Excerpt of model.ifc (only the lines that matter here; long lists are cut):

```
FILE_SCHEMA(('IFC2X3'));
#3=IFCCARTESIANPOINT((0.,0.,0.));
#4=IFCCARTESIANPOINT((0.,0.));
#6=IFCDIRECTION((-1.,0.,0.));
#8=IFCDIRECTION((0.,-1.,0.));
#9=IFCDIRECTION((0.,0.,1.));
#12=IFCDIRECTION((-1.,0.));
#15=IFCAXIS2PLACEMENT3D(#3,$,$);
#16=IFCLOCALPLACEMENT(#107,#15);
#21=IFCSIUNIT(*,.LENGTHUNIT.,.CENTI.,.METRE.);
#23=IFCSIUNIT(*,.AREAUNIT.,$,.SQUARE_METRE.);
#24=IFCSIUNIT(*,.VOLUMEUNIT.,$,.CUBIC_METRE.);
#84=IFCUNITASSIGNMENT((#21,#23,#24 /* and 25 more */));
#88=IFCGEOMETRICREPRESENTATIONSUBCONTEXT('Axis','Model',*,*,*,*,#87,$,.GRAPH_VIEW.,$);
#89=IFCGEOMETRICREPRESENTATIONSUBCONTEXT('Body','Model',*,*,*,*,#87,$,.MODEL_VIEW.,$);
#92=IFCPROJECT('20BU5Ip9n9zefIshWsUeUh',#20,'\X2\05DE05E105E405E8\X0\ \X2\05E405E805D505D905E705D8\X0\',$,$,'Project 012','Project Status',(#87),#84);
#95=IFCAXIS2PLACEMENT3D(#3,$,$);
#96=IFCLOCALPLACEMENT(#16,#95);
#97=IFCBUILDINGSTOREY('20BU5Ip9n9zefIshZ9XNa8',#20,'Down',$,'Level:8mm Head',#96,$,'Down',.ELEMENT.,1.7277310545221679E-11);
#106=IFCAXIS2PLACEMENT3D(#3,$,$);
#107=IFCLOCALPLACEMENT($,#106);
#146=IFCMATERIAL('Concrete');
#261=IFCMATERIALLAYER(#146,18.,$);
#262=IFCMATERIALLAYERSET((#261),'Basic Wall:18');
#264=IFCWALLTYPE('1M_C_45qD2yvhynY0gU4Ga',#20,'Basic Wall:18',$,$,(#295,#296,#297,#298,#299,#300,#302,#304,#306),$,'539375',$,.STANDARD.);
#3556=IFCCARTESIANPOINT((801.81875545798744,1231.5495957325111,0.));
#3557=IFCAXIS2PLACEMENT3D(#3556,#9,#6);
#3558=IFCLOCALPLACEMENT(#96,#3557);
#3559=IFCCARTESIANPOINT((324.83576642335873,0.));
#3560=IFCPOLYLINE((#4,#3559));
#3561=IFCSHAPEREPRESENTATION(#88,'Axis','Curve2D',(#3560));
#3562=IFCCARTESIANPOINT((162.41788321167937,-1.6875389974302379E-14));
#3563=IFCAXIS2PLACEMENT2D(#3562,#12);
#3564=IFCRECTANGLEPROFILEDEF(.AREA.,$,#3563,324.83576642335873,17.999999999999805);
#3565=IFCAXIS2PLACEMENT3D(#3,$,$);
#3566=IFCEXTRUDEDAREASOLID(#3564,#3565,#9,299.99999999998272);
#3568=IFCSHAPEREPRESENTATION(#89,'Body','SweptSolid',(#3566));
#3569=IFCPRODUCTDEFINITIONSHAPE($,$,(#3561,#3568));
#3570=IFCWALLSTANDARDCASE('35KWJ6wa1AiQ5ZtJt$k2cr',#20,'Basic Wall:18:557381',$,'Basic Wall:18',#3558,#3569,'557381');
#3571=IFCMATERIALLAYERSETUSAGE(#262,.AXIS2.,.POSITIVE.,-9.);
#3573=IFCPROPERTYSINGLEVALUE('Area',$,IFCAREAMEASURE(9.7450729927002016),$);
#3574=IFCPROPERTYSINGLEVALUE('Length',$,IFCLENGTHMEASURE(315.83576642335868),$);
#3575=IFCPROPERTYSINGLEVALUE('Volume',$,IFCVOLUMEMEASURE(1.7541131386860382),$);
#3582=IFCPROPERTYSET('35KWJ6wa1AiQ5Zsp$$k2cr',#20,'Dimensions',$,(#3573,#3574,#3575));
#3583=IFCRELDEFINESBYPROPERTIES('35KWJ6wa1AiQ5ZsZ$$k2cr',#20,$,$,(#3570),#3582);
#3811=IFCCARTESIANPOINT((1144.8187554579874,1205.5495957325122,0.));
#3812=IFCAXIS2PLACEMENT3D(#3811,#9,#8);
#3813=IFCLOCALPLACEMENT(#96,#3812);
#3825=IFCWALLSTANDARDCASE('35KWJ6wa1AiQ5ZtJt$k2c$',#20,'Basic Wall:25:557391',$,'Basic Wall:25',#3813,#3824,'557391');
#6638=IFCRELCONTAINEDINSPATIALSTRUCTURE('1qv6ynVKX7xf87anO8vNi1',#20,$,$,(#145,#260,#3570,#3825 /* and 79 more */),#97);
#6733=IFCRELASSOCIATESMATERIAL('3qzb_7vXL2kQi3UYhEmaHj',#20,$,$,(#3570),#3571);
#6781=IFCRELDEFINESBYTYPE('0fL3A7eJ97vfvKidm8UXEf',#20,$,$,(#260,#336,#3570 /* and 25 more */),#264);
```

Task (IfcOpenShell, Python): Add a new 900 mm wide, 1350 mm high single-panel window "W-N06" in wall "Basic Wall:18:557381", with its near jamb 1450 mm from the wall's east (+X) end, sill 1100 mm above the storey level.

```python
import numpy as np
import ifcopenshell
import ifcopenshell.api.feature
import ifcopenshell.api.geometry
import ifcopenshell.api.pset
import ifcopenshell.api.root
import ifcopenshell.api.spatial
import ifcopenshell.api.type
import ifcopenshell.geom
import ifcopenshell.util.element
import ifcopenshell.util.placement
import ifcopenshell.util.representation
import ifcopenshell.util.shape
import ifcopenshell.util.unit

model = ifcopenshell.open("model.ifc")
unit_scale = ifcopenshell.util.unit.calculate_unit_scale(model)
area_scale = ifcopenshell.util.unit.calculate_unit_scale(model, "AREAUNIT")
volume_scale = ifcopenshell.util.unit.calculate_unit_scale(model, "VOLUMEUNIT")
settings = ifcopenshell.geom.settings()


def volume(element):
    """Net volume in cubic metres, openings subtracted."""
    shape = ifcopenshell.geom.create_shape(settings, element)
    return ifcopenshell.util.shape.get_volume(shape.geometry)


wall = model.by_guid("35KWJ6wa1AiQ5ZtJt$k2cr")
storey = ifcopenshell.util.element.get_container(wall, ifc_class="IfcBuildingStorey")
context = ifcopenshell.util.representation.get_context(model, "Model", "Body", "MODEL_VIEW")
before = volume(wall)

width, height, from_end, sill = 0.9, 1.35, 1.45, 1.1  # metres

# The wall runs along its own X axis, and the end named is its -X end.
wall_shape = ifcopenshell.geom.create_shape(settings, wall)
x, y, z = ifcopenshell.util.shape.get_vertices(wall_shape.geometry).T
start = x.min() + from_end
face, thickness = float(y.min()), float(y.max() - y.min())
wall_matrix = ifcopenshell.util.placement.get_local_placement(wall.ObjectPlacement)
level = ifcopenshell.util.placement.get_local_placement(storey.ObjectPlacement)[2, 3]


def in_wall(x, y):
    """Placement at x, y metres in the wall's axes, at sill height."""
    matrix = wall_matrix.copy()
    matrix[:, 3] = wall_matrix @ np.array([x / unit_scale, y / unit_scale, 0.0, 1.0])
    matrix[2, 3] = level + sill / unit_scale
    return matrix


# Opening: a box that overshoots both wall faces by 50 mm.
opening = ifcopenshell.api.root.create_entity(model, ifc_class="IfcOpeningElement")
box = ifcopenshell.api.geometry.add_wall_representation(
    model, context=context, length=width, height=height, thickness=thickness + 0.1
)
ifcopenshell.api.geometry.assign_representation(model, product=opening, representation=box)
ifcopenshell.api.geometry.edit_object_placement(model, product=opening, matrix=in_wall(start, face - 0.05), is_si=False)
ifcopenshell.api.feature.add_feature(model, feature=opening, element=wall)

window = ifcopenshell.api.root.create_entity(model, ifc_class="IfcWindow", name="W-N06")
window.OverallWidth, window.OverallHeight = width / unit_scale, height / unit_scale
body = ifcopenshell.api.geometry.add_window_representation(
    model,
    context=context,
    overall_width=window.OverallWidth,
    overall_height=window.OverallHeight,
    partition_type="SINGLE_PANEL",
)
ifcopenshell.api.geometry.assign_representation(model, product=window, representation=body)
ifcopenshell.api.spatial.assign_container(model, products=[window], relating_structure=storey)
fills = ifcopenshell.api.feature.add_filling(model, opening=opening, element=window)
fills.OwnerHistory = window.OwnerHistory  # required in IFC2X3

# IFC2X3 keeps the operation on the window style.
style = ifcopenshell.api.root.create_entity(model, ifc_class="IfcWindowStyle", name="W-N06")
style.OperationType, style.ConstructionType = "SINGLE_PANEL", "NOTDEFINED"
style.ParameterTakesPrecedence = style.Sizeable = False
ifcopenshell.api.type.assign_type(model, related_objects=[window], relating_type=style)

# Centre the window in the wall's thickness.
ifcopenshell.api.geometry.edit_object_placement(model, product=window, matrix=in_wall(start, face), is_si=False)
window_shape = ifcopenshell.geom.create_shape(settings, window)
depth = ifcopenshell.util.shape.get_vertices(window_shape.geometry)[:, 1]
offset = face + thickness / 2 - (depth.min() + depth.max()) / 2
ifcopenshell.api.geometry.edit_object_placement(model, product=window, matrix=in_wall(start, offset), is_si=False)

after = volume(wall)

# Update the wall's stored quantities.
pset = model.by_id(ifcopenshell.util.element.get_pset(wall, "Dimensions", should_inherit=False)["id"])
ifcopenshell.api.pset.edit_pset(model, pset=pset, properties={
    "Area": model.create_entity("IfcAreaMeasure", after / thickness / area_scale),
    "Volume": model.create_entity("IfcVolumeMeasure", after / volume_scale),
})

print(f"wall volume {before:.3f} -> {after:.3f} m3")

model.write("model_rev.ifc")
```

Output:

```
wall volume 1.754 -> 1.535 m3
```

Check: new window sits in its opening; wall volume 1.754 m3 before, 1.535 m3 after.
